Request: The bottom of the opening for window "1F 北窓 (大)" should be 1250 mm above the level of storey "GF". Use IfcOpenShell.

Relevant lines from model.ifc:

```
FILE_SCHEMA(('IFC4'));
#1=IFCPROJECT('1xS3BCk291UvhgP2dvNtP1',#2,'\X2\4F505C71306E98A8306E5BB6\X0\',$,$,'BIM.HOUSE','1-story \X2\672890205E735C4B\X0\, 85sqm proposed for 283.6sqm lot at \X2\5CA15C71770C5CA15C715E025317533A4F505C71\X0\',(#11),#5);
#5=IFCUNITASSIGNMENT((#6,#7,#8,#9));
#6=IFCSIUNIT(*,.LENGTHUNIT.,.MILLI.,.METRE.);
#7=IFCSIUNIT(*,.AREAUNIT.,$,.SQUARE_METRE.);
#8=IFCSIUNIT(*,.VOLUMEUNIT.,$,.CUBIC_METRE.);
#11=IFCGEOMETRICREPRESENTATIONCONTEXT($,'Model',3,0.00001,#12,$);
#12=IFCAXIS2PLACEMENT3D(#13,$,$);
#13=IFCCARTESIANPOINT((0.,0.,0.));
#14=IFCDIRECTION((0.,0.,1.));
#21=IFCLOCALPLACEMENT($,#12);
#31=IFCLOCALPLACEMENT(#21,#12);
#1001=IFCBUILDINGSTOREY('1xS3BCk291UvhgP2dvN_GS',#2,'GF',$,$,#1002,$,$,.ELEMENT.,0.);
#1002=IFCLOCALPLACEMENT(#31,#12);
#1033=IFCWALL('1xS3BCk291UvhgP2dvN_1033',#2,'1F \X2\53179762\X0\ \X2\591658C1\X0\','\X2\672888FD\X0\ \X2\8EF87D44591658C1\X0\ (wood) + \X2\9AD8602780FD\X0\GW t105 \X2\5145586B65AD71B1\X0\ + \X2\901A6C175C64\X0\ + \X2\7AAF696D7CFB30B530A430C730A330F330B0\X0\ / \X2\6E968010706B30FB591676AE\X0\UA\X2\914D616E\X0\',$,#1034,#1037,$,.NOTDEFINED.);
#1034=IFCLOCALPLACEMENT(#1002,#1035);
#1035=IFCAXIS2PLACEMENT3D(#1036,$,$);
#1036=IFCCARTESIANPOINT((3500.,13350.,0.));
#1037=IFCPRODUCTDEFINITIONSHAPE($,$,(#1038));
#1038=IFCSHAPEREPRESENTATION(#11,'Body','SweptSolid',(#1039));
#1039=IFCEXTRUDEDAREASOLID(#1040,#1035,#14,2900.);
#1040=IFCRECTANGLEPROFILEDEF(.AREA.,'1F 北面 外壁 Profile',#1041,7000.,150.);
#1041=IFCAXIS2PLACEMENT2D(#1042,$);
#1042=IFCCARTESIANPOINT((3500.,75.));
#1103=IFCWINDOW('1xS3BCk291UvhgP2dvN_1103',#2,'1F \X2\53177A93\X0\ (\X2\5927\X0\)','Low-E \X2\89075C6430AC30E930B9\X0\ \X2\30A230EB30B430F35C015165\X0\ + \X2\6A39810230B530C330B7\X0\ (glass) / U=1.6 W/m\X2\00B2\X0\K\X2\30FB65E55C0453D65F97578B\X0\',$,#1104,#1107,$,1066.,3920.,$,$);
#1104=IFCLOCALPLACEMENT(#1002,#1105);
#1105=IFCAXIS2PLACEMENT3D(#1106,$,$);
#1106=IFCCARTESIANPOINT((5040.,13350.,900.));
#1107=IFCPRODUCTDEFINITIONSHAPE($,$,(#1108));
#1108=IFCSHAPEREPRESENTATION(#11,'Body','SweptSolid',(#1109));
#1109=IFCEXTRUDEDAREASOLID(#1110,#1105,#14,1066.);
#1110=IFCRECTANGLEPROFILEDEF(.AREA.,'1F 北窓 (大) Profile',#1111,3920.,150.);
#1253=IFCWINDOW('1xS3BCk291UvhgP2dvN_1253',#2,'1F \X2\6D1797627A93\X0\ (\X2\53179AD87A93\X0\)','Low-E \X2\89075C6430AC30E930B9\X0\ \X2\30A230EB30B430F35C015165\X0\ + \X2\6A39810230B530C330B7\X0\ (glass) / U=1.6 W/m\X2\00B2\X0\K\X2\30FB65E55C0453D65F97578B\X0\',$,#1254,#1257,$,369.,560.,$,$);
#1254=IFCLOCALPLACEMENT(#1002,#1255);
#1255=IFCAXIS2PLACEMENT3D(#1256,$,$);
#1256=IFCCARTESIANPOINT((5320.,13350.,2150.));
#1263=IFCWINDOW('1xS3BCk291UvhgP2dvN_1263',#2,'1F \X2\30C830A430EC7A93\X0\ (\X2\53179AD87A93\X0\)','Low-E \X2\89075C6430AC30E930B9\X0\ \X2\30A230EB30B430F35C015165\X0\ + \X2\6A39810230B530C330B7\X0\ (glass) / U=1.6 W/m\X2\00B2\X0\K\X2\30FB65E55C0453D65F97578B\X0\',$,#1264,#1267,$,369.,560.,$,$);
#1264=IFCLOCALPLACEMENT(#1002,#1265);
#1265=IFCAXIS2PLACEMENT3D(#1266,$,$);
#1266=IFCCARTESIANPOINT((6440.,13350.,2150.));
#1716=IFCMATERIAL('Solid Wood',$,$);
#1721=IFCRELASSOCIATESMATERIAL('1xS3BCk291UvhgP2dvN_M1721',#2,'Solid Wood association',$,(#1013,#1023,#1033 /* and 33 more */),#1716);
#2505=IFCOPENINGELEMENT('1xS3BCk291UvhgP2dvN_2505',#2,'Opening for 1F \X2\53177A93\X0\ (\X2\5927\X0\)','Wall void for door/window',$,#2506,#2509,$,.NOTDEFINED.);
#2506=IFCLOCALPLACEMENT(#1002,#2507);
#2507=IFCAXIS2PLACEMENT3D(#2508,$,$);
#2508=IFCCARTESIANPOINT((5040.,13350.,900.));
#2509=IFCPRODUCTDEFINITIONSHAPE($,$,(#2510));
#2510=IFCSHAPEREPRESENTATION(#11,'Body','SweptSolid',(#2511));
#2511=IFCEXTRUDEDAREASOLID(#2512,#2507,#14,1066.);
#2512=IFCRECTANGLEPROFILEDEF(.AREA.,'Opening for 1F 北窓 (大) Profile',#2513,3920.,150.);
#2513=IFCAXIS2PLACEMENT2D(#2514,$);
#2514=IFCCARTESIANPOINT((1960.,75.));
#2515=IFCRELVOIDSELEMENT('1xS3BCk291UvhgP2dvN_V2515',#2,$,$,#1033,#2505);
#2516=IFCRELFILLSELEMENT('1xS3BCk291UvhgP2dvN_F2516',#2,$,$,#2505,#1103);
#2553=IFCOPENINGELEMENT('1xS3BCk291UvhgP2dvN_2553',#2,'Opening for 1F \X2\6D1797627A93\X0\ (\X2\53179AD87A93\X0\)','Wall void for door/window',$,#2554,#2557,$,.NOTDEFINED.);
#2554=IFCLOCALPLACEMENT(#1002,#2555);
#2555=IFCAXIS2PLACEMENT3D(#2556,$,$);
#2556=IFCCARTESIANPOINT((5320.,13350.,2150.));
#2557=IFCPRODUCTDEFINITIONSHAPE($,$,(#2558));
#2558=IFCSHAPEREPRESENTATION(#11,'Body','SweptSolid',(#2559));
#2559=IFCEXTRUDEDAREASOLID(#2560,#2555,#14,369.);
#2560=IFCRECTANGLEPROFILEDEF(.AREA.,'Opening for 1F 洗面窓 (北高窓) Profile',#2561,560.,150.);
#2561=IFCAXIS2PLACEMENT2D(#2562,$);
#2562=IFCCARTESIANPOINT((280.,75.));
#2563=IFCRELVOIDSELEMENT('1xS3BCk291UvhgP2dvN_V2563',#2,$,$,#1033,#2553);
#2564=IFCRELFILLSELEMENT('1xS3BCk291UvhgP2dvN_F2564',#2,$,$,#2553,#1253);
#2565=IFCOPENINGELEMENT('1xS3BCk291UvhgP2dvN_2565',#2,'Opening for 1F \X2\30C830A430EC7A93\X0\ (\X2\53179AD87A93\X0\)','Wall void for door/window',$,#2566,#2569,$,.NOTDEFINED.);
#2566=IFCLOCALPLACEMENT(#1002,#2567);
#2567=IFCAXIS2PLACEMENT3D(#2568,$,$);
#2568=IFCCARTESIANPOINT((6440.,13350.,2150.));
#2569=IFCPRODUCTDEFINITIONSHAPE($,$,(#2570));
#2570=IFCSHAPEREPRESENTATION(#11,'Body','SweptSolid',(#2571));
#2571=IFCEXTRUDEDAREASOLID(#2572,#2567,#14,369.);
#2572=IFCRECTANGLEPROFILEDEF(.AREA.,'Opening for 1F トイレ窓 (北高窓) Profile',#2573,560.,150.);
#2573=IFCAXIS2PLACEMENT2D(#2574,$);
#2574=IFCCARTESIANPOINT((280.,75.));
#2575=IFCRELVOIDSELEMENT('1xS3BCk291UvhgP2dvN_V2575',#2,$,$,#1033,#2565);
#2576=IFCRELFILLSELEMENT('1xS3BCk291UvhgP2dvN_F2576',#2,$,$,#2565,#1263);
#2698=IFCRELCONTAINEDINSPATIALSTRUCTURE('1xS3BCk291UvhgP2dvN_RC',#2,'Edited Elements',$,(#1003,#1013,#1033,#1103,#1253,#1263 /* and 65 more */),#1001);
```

```python
import numpy as np
import ifcopenshell
import ifcopenshell.api.geometry
import ifcopenshell.geom
import ifcopenshell.util.element
import ifcopenshell.util.placement
import ifcopenshell.util.shape
import ifcopenshell.util.unit

model = ifcopenshell.open("model.ifc")
unit_scale = ifcopenshell.util.unit.calculate_unit_scale(model)

window = model.by_guid("1xS3BCk291UvhgP2dvN_1103")
opening = window.FillsVoids[0].RelatingOpeningElement
storey = ifcopenshell.util.element.get_container(window, ifc_class="IfcBuildingStorey")
level = ifcopenshell.util.placement.get_local_placement(storey.ObjectPlacement)[2, 3]

# The opening's origin need not be at the sill, so measure its lowest point.
shape = ifcopenshell.geom.create_shape(ifcopenshell.geom.settings(), opening)
bottom = ifcopenshell.util.shape.get_shape_bottom_elevation(shape, shape.geometry) / unit_scale
dz = level + 1250.0 - bottom

shift = np.array([0.0, 0.0, dz])
# The window is not placed relative to its opening, so move both.
for product in (opening, window):
    matrix = ifcopenshell.util.placement.get_local_placement(product.ObjectPlacement)
    matrix[:3, 3] += shift
    ifcopenshell.api.geometry.edit_object_placement(model, product=product, matrix=matrix, is_si=False)

print(f"moved by {dz * unit_scale:+.3f} m")

model.write("model-out.ifc")
```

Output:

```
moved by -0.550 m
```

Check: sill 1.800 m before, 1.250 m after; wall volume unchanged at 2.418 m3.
